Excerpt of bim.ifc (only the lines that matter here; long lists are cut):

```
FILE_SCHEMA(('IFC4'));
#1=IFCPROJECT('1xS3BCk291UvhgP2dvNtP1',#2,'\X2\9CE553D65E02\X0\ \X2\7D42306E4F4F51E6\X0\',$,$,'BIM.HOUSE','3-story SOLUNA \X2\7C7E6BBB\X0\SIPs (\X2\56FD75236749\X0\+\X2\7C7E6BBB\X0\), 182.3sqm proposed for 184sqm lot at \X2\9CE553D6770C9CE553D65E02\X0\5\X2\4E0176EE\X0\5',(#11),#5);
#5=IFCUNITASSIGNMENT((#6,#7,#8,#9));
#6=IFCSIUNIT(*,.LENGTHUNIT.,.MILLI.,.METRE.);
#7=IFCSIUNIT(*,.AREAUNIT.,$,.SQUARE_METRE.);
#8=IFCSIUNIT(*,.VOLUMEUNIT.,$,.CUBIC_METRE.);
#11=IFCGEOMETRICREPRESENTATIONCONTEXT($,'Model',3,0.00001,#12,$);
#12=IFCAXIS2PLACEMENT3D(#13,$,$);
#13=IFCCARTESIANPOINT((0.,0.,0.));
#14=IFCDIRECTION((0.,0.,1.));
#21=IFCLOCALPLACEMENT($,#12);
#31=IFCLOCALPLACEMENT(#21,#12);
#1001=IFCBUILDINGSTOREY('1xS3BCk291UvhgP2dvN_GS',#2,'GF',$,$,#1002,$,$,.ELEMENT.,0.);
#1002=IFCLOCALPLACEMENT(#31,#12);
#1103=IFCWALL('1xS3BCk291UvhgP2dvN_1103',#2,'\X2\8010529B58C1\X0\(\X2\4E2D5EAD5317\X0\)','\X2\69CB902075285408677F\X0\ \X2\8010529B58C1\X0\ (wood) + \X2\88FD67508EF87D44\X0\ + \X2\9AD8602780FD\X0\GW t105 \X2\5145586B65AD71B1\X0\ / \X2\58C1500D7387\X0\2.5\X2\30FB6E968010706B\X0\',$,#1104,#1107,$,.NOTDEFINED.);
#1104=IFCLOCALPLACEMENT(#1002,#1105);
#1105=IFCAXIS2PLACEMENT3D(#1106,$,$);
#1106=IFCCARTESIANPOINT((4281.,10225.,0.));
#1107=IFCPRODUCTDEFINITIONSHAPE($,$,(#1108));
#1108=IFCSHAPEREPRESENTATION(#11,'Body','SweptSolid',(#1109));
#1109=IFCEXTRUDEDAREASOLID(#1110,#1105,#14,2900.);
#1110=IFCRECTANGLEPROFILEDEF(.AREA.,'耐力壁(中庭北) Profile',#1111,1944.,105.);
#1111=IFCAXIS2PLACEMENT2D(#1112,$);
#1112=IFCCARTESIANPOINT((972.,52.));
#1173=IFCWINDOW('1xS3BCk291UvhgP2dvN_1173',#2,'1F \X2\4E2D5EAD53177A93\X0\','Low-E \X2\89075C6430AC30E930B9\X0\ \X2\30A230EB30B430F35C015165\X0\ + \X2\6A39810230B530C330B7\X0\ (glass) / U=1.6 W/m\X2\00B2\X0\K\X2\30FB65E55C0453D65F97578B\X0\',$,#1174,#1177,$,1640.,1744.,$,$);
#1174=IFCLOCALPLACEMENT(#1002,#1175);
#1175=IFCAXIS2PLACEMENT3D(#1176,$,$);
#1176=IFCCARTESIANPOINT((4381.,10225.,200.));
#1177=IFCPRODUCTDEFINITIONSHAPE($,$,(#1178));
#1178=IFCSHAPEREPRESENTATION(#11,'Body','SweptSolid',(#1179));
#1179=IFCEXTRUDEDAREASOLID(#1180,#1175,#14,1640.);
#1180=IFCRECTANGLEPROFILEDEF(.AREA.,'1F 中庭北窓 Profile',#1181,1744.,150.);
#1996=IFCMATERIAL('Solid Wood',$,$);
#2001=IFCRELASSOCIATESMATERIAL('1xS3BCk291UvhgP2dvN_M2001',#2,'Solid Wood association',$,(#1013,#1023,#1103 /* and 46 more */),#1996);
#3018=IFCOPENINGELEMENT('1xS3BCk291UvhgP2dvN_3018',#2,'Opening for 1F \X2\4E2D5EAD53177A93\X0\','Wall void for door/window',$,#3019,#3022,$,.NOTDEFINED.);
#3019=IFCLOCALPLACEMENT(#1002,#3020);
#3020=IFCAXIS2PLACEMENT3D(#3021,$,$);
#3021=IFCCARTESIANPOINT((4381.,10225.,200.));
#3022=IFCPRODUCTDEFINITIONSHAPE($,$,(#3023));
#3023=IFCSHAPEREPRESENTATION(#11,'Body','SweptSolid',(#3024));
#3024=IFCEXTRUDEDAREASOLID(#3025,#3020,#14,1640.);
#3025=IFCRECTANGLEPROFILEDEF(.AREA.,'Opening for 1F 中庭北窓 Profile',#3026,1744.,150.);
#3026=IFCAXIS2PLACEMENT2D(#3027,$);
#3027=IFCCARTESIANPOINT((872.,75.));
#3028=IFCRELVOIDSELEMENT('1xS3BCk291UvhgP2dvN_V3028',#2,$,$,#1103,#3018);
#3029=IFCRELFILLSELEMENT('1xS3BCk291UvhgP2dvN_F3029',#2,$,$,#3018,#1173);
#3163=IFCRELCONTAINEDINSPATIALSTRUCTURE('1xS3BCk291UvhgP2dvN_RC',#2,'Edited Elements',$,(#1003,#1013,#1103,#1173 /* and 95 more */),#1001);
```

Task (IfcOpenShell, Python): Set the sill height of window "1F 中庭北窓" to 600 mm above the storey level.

```python
import numpy as np
import ifcopenshell
import ifcopenshell.api.geometry
import ifcopenshell.geom
import ifcopenshell.util.element
import ifcopenshell.util.placement
import ifcopenshell.util.shape
import ifcopenshell.util.unit

model = ifcopenshell.open("bim.ifc")
unit_scale = ifcopenshell.util.unit.calculate_unit_scale(model)

window = model.by_guid("1xS3BCk291UvhgP2dvN_1173")
opening = window.FillsVoids[0].RelatingOpeningElement
storey = ifcopenshell.util.element.get_container(window, ifc_class="IfcBuildingStorey")
level = ifcopenshell.util.placement.get_local_placement(storey.ObjectPlacement)[2, 3]

# The opening's origin need not be at the sill, so measure its lowest point.
shape = ifcopenshell.geom.create_shape(ifcopenshell.geom.settings(), opening)
bottom = ifcopenshell.util.shape.get_shape_bottom_elevation(shape, shape.geometry) / unit_scale
dz = level + 600.0 - bottom

shift = np.array([0.0, 0.0, dz])
# The window is not placed relative to its opening, so move both.
for product in (opening, window):
    matrix = ifcopenshell.util.placement.get_local_placement(product.ObjectPlacement)
    matrix[:3, 3] += shift
    ifcopenshell.api.geometry.edit_object_placement(model, product=product, matrix=matrix, is_si=False)

print(f"moved by {dz * unit_scale:+.3f} m")

model.write("bim_v2.ifc")
```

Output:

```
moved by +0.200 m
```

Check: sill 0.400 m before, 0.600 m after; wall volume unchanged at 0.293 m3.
